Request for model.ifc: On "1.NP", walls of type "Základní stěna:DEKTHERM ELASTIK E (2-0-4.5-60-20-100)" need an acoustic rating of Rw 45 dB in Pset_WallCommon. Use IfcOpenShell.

First a look at what the model holds.

```python
import ifcopenshell
import ifcopenshell.util.element

model = ifcopenshell.open("model.ifc")
print(model.schema)
storey = next(s for s in model.by_type("IfcBuildingStorey") if s.Name == "1.NP")
walls = [e for e in ifcopenshell.util.element.get_decomposition(storey) if e.is_a("IfcWall")]
seen = {}
for e in walls:
    element_type = ifcopenshell.util.element.get_type(e)
    key = (element_type.Name if element_type != e and element_type else None, ifcopenshell.util.element.get_pset(e, "Pset_WallCommon", "AcousticRating"))
    seen[key] = seen.get(key, 0) + 1
for (name, value), count in sorted(seen.items(), key=str):
    print(count, "x", name, "|", value)
```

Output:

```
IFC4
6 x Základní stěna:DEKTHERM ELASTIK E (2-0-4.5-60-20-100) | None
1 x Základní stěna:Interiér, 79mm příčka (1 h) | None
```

```python
import ifcopenshell
import ifcopenshell.api.pset
import ifcopenshell.util.element

model = ifcopenshell.open("model.ifc")

storey = next(s for s in model.by_type("IfcBuildingStorey") if s.Name == "1.NP")
walls = [e for e in ifcopenshell.util.element.get_decomposition(storey) if e.is_a("IfcWall")]

count = 0
for e in walls:
    element_type = ifcopenshell.util.element.get_type(e)
    if element_type in (None, e) or element_type.Name != "Základní stěna:DEKTHERM ELASTIK E (2-0-4.5-60-20-100)":
        continue
    # add_pset returns the element's existing set when there is one.
    pset = ifcopenshell.api.pset.add_pset(model, product=e, name="Pset_WallCommon")
    ifcopenshell.api.pset.edit_pset(model, pset=pset, properties={"AcousticRating": "Rw 45 dB"})
    count += 1

print(count, "walls updated")

model.write("model_updated.ifc")
```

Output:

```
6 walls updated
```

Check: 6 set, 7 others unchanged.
